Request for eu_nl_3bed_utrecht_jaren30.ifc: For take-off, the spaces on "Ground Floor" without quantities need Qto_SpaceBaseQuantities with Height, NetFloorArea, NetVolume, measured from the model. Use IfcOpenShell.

First a look at what the model holds.

```python
import ifcopenshell
import ifcopenshell.util.element
import ifcopenshell.util.unit

model = ifcopenshell.open("eu_nl_3bed_utrecht_jaren30.ifc")
print(model.schema)
for unit_type in ("LENGTHUNIT", "AREAUNIT", "VOLUMEUNIT"):
    print(unit_type, ifcopenshell.util.unit.calculate_unit_scale(model, unit_type))
storey = next(s for s in model.by_type("IfcBuildingStorey") if s.Name == "Ground Floor")
spaces = [e for e in ifcopenshell.util.element.get_decomposition(storey) if e.is_a("IfcSpace")]
for e in sorted(spaces, key=lambda e: e.id()):
    print(e.id(), e.is_a(), e.Name, list(ifcopenshell.util.element.get_psets(e, qtos_only=True)), sep=" | ")
```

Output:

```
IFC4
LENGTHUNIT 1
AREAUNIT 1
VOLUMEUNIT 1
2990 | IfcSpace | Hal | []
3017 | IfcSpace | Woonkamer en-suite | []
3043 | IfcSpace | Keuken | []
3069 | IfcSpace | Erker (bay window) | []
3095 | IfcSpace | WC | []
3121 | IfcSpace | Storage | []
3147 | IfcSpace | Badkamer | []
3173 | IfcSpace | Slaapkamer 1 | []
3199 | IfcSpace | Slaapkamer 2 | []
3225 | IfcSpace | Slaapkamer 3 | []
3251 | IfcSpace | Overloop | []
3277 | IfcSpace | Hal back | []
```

```python
import ifcopenshell
import ifcopenshell.api.pset
import ifcopenshell.geom
import ifcopenshell.util.element
import ifcopenshell.util.shape
import ifcopenshell.util.unit

model = ifcopenshell.open("eu_nl_3bed_utrecht_jaren30.ifc")
unit_scale = ifcopenshell.util.unit.calculate_unit_scale(model)
area_scale = ifcopenshell.util.unit.calculate_unit_scale(model, "AREAUNIT")
volume_scale = ifcopenshell.util.unit.calculate_unit_scale(model, "VOLUMEUNIT")
settings = ifcopenshell.geom.settings()

storey = next(s for s in model.by_type("IfcBuildingStorey") if s.Name == "Ground Floor")
spaces = [e for e in ifcopenshell.util.element.get_decomposition(storey) if e.is_a("IfcSpace")]

for e in sorted(spaces, key=lambda e: e.id()):
    if ifcopenshell.util.element.get_psets(e, qtos_only=True, should_inherit=False):
        continue
    # Geometry comes back in metres, in the element's own axes.
    shape = ifcopenshell.geom.create_shape(settings, e)
    values = {
        "Height": ifcopenshell.util.shape.get_z(shape.geometry) / unit_scale,
        "NetFloorArea": ifcopenshell.util.shape.get_footprint_area(shape.geometry) / area_scale,
        "NetVolume": ifcopenshell.util.shape.get_volume(shape.geometry) / volume_scale,
    }
    qto = ifcopenshell.api.pset.add_qto(model, product=e, name="Qto_SpaceBaseQuantities")
    ifcopenshell.api.pset.edit_qto(model, qto=qto, properties=values)
    print(e.id(), {k: round(v, 3) for k, v in values.items()})

model.write("eu_nl_3bed_utrecht_jaren30_rev.ifc")
```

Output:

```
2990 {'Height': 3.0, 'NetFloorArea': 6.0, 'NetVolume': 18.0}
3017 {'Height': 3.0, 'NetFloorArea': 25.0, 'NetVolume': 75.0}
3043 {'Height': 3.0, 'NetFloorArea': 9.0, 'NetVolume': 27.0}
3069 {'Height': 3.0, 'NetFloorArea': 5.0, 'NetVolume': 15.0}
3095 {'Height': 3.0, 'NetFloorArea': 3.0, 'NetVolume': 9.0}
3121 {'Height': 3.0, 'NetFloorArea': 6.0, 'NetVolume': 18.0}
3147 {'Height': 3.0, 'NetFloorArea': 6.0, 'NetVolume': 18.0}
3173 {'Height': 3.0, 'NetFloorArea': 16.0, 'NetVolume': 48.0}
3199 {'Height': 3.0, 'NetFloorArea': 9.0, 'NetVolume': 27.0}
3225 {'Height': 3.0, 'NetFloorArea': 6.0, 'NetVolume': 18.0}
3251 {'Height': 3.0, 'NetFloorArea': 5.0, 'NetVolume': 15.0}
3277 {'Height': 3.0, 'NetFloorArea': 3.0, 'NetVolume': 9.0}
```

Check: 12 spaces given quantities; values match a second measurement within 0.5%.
